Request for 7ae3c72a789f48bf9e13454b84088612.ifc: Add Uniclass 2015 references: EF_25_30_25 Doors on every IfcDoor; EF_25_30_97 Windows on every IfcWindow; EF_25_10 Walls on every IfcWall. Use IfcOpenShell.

First a look at what the model holds.

```python
import ifcopenshell

model = ifcopenshell.open("7ae3c72a789f48bf9e13454b84088612.ifc")
print(model.schema)
print("classifications:", [c.Name for c in model.by_type("IfcClassification")])
for ifc_class in ("IfcDoor", "IfcRoof", "IfcStair", "IfcWall", "IfcWindow"):
    print(ifc_class, len(model.by_type(ifc_class)))
```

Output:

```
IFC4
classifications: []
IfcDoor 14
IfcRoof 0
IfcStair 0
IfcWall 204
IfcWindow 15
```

```python
import ifcopenshell
import ifcopenshell.api.classification

model = ifcopenshell.open("7ae3c72a789f48bf9e13454b84088612.ifc")

system = ifcopenshell.api.classification.add_classification(model, classification="Uniclass 2015")

codes = {
    "IfcDoor": ("EF_25_30_25", "Doors"),
    "IfcWindow": ("EF_25_30_97", "Windows"),
    "IfcWall": ("EF_25_10", "Walls"),
}
for ifc_class, (code, name) in codes.items():
    products = model.by_type(ifc_class)
    ifcopenshell.api.classification.add_reference(
        model, products=products, classification=system, identification=code, name=name
    )
    print(code, len(products))

model.write("7ae3c72a789f48bf9e13454b84088612_rev.ifc")
```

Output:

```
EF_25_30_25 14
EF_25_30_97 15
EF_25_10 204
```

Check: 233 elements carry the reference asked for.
